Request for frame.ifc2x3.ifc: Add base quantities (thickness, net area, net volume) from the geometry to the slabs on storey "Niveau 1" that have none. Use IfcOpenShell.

First a look at what the model holds.

```python
import ifcopenshell
import ifcopenshell.util.element
import ifcopenshell.util.unit

model = ifcopenshell.open("frame.ifc2x3.ifc")
print(model.schema)
for unit_type in ("LENGTHUNIT", "AREAUNIT", "VOLUMEUNIT"):
    print(unit_type, ifcopenshell.util.unit.calculate_unit_scale(model, unit_type))
storey = next(s for s in model.by_type("IfcBuildingStorey") if s.Name == "Niveau 1")
slabs = [e for e in ifcopenshell.util.element.get_decomposition(storey) if e.is_a("IfcSlab")]
for e in sorted(slabs, key=lambda e: e.id()):
    print(e.id(), e.is_a(), e.Name, list(ifcopenshell.util.element.get_psets(e, qtos_only=True)), sep=" | ")
```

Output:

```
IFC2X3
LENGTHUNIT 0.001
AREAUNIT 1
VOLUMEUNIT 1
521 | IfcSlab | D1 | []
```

```python
import ifcopenshell
import ifcopenshell.api.pset
import ifcopenshell.geom
import ifcopenshell.util.element
import ifcopenshell.util.shape
import ifcopenshell.util.unit

model = ifcopenshell.open("frame.ifc2x3.ifc")
unit_scale = ifcopenshell.util.unit.calculate_unit_scale(model)
area_scale = ifcopenshell.util.unit.calculate_unit_scale(model, "AREAUNIT")
volume_scale = ifcopenshell.util.unit.calculate_unit_scale(model, "VOLUMEUNIT")
settings = ifcopenshell.geom.settings()

storey = next(s for s in model.by_type("IfcBuildingStorey") if s.Name == "Niveau 1")
slabs = [e for e in ifcopenshell.util.element.get_decomposition(storey) if e.is_a("IfcSlab")]

for e in sorted(slabs, key=lambda e: e.id()):
    if ifcopenshell.util.element.get_psets(e, qtos_only=True, should_inherit=False):
        continue
    # Geometry comes back in metres, in the element's own axes.
    shape = ifcopenshell.geom.create_shape(settings, e)
    values = {
        "Width": ifcopenshell.util.shape.get_z(shape.geometry) / unit_scale,
        "NetArea": ifcopenshell.util.shape.get_footprint_area(shape.geometry) / area_scale,
        "NetVolume": ifcopenshell.util.shape.get_volume(shape.geometry) / volume_scale,
    }
    qto = ifcopenshell.api.pset.add_qto(model, product=e, name="BaseQuantities")
    ifcopenshell.api.pset.edit_qto(model, qto=qto, properties=values)
    print(e.id(), {k: round(v, 3) for k, v in values.items()})

model.write("frame.ifc2x3_rev.ifc")
```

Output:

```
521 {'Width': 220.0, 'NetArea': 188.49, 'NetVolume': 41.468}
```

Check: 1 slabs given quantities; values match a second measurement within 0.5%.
